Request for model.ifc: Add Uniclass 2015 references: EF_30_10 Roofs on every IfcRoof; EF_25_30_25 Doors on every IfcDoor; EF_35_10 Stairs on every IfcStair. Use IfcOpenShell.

First a look at what the model holds.

```python
import ifcopenshell

model = ifcopenshell.open("model.ifc")
print(model.schema)
print("classifications:", [c.Name for c in model.by_type("IfcClassification")])
for ifc_class in ("IfcDoor", "IfcRoof", "IfcStair", "IfcWall", "IfcWindow"):
    print(ifc_class, len(model.by_type(ifc_class)))
```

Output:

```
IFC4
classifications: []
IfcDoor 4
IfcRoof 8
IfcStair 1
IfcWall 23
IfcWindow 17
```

```python
import ifcopenshell
import ifcopenshell.api.classification

model = ifcopenshell.open("model.ifc")

system = ifcopenshell.api.classification.add_classification(model, classification="Uniclass 2015")

codes = {
    "IfcRoof": ("EF_30_10", "Roofs"),
    "IfcDoor": ("EF_25_30_25", "Doors"),
    "IfcStair": ("EF_35_10", "Stairs"),
}
for ifc_class, (code, name) in codes.items():
    products = model.by_type(ifc_class)
    ifcopenshell.api.classification.add_reference(
        model, products=products, classification=system, identification=code, name=name
    )
    print(code, len(products))

model.write("model_rev.ifc")
```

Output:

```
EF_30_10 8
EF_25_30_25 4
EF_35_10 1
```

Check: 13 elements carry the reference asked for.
